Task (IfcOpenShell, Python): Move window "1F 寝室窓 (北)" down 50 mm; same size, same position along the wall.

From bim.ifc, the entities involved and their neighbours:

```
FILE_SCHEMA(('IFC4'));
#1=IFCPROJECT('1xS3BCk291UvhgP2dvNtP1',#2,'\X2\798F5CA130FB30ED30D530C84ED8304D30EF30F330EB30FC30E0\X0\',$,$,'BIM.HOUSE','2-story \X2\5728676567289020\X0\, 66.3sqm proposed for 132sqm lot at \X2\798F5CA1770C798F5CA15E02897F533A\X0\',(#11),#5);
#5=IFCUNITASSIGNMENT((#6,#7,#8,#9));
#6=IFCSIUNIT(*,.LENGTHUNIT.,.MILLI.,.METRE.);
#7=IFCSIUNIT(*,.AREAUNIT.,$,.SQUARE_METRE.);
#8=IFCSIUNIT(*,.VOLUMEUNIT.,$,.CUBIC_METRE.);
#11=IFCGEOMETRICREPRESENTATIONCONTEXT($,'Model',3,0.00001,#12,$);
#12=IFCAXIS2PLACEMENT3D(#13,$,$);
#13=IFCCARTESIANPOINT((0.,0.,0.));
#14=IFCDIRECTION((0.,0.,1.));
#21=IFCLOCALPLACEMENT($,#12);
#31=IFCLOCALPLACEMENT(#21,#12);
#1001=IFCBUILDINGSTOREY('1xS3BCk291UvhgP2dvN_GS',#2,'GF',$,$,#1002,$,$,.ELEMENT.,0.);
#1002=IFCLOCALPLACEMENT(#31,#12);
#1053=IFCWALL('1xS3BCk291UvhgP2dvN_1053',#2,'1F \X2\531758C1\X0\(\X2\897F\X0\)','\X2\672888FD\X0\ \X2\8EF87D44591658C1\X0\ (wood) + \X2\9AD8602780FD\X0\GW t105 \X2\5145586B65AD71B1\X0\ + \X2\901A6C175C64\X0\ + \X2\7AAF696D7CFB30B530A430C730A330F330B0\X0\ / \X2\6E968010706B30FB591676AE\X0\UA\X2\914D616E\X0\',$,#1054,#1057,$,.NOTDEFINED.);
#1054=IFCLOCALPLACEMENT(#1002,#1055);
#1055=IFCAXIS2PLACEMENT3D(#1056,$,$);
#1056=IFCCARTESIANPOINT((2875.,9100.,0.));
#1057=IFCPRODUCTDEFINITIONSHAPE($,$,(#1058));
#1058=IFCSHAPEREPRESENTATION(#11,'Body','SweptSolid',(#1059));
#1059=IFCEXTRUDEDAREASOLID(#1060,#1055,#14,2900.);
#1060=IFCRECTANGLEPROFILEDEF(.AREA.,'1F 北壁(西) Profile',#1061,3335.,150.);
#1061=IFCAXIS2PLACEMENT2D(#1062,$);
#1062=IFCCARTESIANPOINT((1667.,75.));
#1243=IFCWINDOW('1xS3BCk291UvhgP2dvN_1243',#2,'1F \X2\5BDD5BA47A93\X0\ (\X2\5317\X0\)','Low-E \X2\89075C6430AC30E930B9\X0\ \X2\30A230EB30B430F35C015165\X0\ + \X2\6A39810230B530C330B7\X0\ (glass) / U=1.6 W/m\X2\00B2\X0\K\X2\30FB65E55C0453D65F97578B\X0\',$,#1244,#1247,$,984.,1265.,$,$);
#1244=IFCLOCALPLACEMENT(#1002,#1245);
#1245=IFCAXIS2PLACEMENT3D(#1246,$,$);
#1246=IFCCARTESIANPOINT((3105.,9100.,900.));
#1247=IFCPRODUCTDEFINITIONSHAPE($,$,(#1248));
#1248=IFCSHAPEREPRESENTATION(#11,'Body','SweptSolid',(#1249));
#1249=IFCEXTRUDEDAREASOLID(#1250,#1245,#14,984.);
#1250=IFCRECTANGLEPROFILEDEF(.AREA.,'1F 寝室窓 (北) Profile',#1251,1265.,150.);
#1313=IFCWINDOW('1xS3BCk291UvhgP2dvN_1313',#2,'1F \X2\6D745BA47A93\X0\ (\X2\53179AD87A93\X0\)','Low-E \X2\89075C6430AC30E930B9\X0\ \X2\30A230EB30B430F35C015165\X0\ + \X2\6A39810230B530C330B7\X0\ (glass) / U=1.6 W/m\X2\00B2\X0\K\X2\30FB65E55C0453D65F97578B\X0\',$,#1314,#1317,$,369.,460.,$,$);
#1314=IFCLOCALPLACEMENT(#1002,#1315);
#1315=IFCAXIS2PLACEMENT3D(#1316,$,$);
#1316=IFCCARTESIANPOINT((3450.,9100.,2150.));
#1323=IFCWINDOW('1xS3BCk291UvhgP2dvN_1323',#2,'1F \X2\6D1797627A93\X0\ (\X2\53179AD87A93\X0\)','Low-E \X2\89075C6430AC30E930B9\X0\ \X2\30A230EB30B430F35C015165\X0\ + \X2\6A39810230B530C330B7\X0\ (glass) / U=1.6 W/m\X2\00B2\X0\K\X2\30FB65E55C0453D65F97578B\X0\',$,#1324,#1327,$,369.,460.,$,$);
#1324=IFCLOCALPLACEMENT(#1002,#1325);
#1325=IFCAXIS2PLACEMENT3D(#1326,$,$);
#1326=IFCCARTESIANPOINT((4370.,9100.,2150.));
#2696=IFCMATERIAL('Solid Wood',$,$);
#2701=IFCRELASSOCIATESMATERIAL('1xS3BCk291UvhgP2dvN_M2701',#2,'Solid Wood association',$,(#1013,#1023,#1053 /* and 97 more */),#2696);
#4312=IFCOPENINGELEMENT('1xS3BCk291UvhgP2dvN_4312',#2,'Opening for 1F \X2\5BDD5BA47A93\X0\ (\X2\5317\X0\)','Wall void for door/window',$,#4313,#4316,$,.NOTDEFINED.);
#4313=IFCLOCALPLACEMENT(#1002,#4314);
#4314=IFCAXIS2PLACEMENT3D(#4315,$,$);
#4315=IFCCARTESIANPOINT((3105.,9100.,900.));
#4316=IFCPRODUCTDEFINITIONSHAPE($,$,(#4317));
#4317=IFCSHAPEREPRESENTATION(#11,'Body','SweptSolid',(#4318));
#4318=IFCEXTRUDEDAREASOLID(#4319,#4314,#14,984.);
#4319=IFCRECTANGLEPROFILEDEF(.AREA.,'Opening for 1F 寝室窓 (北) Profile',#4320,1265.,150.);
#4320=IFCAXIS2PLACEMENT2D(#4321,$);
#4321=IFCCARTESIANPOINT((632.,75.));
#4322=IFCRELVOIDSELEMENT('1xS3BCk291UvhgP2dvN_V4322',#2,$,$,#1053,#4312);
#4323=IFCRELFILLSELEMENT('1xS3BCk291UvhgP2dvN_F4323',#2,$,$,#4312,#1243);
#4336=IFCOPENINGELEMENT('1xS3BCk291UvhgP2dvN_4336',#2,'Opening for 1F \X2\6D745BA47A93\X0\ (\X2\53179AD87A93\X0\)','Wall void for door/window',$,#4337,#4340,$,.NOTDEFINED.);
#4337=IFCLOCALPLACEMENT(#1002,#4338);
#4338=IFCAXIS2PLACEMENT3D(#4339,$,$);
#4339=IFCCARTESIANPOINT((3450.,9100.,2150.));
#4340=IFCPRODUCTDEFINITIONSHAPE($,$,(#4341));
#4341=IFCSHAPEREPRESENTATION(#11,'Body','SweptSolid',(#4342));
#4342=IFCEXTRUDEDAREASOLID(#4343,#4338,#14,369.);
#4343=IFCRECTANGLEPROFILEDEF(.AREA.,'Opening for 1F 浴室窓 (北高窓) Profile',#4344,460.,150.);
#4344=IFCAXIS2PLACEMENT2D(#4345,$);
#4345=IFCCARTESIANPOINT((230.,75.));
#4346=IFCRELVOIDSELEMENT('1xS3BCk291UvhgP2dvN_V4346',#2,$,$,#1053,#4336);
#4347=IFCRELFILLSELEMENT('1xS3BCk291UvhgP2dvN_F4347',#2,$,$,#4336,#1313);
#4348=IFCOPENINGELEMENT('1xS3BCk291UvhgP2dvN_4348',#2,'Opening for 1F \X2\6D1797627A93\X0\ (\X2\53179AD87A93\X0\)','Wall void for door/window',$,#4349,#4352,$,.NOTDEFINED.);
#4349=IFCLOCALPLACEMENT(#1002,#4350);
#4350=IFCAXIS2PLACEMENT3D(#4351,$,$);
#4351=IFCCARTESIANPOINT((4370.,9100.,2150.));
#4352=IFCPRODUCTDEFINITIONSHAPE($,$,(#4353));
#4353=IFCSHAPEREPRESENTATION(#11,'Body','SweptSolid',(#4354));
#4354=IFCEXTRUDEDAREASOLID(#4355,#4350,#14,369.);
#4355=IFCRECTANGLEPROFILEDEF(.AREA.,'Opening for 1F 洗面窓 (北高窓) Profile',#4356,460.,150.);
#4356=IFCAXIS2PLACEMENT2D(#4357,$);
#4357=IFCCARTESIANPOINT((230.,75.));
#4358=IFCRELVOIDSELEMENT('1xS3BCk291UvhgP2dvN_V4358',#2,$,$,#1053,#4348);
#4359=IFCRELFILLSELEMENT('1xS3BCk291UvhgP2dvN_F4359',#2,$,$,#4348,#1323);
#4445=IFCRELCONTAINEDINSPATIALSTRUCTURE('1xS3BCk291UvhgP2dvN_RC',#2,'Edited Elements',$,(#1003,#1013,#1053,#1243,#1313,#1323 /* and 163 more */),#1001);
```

```python
import numpy as np
import ifcopenshell
import ifcopenshell.api.geometry
import ifcopenshell.util.placement
import ifcopenshell.util.unit

model = ifcopenshell.open("bim.ifc")
unit_scale = ifcopenshell.util.unit.calculate_unit_scale(model)

window = model.by_id(1243)
opening = window.FillsVoids[0].RelatingOpeningElement
dz = -0.05 / unit_scale

shift = np.array([0.0, 0.0, dz])
# The window is not placed relative to its opening, so move both.
for product in (opening, window):
    matrix = ifcopenshell.util.placement.get_local_placement(product.ObjectPlacement)
    matrix[:3, 3] += shift
    ifcopenshell.api.geometry.edit_object_placement(model, product=product, matrix=matrix, is_si=False)

print(f"moved by {dz * unit_scale:+.3f} m")

model.write("bim_rev.ifc")
```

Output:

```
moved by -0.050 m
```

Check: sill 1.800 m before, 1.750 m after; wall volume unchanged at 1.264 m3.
